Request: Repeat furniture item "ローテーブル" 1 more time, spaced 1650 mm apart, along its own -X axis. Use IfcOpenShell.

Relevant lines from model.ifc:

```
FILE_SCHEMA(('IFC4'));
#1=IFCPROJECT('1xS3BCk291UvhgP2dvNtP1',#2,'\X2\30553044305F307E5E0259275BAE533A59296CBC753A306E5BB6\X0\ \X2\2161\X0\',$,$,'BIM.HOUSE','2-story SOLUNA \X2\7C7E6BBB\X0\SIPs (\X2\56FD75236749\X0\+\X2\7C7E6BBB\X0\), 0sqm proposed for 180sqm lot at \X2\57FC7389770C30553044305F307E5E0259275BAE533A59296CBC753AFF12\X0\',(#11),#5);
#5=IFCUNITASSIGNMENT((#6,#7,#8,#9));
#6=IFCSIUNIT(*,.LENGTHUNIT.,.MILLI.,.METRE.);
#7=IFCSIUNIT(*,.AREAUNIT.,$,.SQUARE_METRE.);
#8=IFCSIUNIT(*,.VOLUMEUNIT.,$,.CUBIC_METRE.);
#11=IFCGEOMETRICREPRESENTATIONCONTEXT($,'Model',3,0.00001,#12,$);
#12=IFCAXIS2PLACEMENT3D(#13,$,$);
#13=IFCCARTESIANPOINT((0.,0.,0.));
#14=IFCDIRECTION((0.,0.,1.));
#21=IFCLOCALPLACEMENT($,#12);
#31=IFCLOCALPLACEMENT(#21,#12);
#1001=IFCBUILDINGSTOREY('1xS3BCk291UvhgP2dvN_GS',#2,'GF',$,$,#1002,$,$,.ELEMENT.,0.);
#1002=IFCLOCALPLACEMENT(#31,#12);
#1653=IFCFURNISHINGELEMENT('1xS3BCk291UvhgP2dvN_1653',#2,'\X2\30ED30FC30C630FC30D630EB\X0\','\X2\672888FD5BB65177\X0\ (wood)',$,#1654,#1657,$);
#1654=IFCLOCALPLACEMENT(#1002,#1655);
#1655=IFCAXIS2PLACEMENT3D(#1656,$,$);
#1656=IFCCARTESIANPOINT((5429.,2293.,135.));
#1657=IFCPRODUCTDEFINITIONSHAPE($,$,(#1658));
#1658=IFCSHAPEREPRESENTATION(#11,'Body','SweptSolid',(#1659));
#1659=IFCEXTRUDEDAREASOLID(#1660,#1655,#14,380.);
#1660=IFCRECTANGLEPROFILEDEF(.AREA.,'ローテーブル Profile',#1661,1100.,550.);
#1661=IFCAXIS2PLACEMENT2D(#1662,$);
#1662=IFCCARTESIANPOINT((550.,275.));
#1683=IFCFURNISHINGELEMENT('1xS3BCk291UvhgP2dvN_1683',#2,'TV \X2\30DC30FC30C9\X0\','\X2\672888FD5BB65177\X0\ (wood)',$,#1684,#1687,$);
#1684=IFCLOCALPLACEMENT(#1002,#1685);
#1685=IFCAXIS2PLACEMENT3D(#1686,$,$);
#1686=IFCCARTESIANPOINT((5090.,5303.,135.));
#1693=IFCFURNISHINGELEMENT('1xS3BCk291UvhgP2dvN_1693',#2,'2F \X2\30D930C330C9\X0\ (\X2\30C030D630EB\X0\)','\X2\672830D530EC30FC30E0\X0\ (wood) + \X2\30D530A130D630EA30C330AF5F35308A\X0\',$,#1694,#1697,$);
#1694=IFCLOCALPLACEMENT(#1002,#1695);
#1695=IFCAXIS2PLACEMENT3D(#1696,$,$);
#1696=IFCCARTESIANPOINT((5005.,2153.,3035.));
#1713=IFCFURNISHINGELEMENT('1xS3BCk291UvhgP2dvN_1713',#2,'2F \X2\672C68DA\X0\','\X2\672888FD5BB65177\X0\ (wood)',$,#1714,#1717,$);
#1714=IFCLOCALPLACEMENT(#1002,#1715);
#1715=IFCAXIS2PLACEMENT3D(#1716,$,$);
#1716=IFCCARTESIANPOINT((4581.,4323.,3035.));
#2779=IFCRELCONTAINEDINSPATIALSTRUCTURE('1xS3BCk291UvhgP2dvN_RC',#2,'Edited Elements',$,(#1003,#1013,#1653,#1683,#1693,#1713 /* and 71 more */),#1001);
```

```python
import ifcopenshell
import ifcopenshell.api.geometry
import ifcopenshell.api.root
import ifcopenshell.util.element
import ifcopenshell.util.placement

model = ifcopenshell.open("model.ifc")


def reuse_history(source, copy):
    """copy_class also copies each property set's owner history, people and application; keep the originals."""
    for rel in copy.IsDefinedBy:
        if rel.is_a("IfcRelDefinesByProperties") and (history := rel.RelatingPropertyDefinition.OwnerHistory):
            rel.RelatingPropertyDefinition.OwnerHistory = source.OwnerHistory
            ifcopenshell.util.element.remove_deep2(model, history)


source = model.by_guid("1xS3BCk291UvhgP2dvN_1653")
base = ifcopenshell.util.placement.get_local_placement(source.ObjectPlacement)
step = -base[:3, 0] * 1650.0

for i in range(1, 2):
    copy = ifcopenshell.api.root.copy_class(model, product=source)
    copy.Representation = ifcopenshell.util.element.copy_deep(
        model, source.Representation, exclude=["IfcGeometricRepresentationContext", "IfcRepresentationMap"]
    )
    reuse_history(source, copy)
    matrix = base.copy()
    matrix[:3, 3] += i * step
    print("added at", matrix[:3, 3].round(3) + 0.0)
    ifcopenshell.api.geometry.edit_object_placement(model, product=copy, matrix=matrix, is_si=False)

model.write("model_v2.ifc")
```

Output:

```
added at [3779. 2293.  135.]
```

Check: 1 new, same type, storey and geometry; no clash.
